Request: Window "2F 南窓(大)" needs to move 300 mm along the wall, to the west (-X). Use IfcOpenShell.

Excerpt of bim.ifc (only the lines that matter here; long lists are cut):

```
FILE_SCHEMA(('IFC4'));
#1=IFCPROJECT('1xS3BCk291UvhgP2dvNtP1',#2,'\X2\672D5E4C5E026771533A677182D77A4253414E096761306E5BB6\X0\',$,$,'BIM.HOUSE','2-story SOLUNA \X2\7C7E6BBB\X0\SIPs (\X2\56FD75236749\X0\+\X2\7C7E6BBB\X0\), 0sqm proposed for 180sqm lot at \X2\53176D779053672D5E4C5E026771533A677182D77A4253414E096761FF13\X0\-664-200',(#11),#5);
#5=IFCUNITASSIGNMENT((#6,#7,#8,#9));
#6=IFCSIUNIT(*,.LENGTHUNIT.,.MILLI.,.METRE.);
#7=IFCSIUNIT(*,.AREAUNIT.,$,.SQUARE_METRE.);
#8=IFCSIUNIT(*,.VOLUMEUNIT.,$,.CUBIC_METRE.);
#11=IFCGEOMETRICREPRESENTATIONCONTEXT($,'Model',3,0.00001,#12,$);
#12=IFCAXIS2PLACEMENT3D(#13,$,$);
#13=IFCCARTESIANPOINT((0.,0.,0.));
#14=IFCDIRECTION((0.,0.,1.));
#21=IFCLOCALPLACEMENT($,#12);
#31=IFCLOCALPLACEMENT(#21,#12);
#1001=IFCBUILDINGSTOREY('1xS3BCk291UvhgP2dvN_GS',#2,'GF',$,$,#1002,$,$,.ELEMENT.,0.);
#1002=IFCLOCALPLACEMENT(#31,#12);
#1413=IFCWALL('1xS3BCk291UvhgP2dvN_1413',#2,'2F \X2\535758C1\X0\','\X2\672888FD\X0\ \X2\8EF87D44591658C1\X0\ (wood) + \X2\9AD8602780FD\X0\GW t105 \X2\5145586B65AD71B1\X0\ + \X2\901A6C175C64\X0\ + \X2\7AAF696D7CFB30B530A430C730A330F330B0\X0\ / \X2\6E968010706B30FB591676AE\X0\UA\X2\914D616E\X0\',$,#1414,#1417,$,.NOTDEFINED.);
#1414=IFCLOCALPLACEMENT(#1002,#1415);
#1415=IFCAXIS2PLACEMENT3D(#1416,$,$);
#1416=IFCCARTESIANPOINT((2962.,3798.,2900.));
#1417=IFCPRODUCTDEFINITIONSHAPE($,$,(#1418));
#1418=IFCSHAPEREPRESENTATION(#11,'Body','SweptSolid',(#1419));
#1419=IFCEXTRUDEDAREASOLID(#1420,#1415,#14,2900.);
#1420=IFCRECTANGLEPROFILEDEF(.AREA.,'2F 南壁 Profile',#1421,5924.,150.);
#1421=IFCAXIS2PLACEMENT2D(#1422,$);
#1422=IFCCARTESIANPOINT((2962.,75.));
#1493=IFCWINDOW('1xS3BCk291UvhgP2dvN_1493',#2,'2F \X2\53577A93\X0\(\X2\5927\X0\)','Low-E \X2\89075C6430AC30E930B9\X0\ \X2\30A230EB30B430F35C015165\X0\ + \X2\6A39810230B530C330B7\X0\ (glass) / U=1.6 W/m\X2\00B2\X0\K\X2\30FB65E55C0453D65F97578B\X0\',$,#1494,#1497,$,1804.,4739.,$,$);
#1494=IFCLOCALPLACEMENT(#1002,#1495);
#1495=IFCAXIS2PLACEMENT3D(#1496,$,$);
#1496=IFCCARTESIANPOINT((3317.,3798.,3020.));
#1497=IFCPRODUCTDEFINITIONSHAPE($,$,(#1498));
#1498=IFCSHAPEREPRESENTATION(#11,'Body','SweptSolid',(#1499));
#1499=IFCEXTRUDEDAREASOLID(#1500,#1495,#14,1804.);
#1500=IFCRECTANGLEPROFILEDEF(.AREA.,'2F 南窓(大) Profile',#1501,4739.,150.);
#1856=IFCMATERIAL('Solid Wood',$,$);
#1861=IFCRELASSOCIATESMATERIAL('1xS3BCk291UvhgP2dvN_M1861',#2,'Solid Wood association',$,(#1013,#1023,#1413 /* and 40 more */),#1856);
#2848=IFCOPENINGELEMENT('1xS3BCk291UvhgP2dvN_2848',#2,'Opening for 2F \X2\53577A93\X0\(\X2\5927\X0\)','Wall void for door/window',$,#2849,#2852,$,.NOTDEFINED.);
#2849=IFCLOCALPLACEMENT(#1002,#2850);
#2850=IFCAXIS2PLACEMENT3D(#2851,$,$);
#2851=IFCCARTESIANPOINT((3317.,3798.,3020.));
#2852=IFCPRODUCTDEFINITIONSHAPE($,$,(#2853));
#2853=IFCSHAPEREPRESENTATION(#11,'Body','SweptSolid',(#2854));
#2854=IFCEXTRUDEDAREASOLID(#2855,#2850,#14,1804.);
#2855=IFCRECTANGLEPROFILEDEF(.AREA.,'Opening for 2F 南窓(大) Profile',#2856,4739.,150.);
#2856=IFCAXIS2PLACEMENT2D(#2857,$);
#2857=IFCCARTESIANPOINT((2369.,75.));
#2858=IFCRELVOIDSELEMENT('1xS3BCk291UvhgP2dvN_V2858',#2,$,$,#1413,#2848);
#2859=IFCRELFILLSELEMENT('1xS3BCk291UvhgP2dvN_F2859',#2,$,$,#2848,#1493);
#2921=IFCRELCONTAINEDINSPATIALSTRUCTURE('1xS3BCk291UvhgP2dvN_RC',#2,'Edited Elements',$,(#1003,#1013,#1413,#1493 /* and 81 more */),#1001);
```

```python
import ifcopenshell
import ifcopenshell.api.geometry
import ifcopenshell.util.placement
import ifcopenshell.util.unit

model = ifcopenshell.open("bim.ifc")
unit_scale = ifcopenshell.util.unit.calculate_unit_scale(model)

window = model.by_guid("1xS3BCk291UvhgP2dvN_1493")
opening = window.FillsVoids[0].RelatingOpeningElement
wall = opening.VoidsElements[0].RelatingBuildingElement

wall_matrix = ifcopenshell.util.placement.get_local_placement(wall.ObjectPlacement)
shift = wall_matrix[:3, 0] * -0.3 / unit_scale
before = ifcopenshell.util.placement.get_local_placement(window.ObjectPlacement)[:3, 3].copy()

# The window is not placed relative to its opening, so move both.
for product in (opening, window):
    matrix = ifcopenshell.util.placement.get_local_placement(product.ObjectPlacement)
    matrix[:3, 3] += shift
    ifcopenshell.api.geometry.edit_object_placement(model, product=product, matrix=matrix, is_si=False)

after = ifcopenshell.util.placement.get_local_placement(window.ObjectPlacement)[:3, 3]
print("window moved by", (after - before).round(3) + 0.0)

model.write("bim-out.ifc")
```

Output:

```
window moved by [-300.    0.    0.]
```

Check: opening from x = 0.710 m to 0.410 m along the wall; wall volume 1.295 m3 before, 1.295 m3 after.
